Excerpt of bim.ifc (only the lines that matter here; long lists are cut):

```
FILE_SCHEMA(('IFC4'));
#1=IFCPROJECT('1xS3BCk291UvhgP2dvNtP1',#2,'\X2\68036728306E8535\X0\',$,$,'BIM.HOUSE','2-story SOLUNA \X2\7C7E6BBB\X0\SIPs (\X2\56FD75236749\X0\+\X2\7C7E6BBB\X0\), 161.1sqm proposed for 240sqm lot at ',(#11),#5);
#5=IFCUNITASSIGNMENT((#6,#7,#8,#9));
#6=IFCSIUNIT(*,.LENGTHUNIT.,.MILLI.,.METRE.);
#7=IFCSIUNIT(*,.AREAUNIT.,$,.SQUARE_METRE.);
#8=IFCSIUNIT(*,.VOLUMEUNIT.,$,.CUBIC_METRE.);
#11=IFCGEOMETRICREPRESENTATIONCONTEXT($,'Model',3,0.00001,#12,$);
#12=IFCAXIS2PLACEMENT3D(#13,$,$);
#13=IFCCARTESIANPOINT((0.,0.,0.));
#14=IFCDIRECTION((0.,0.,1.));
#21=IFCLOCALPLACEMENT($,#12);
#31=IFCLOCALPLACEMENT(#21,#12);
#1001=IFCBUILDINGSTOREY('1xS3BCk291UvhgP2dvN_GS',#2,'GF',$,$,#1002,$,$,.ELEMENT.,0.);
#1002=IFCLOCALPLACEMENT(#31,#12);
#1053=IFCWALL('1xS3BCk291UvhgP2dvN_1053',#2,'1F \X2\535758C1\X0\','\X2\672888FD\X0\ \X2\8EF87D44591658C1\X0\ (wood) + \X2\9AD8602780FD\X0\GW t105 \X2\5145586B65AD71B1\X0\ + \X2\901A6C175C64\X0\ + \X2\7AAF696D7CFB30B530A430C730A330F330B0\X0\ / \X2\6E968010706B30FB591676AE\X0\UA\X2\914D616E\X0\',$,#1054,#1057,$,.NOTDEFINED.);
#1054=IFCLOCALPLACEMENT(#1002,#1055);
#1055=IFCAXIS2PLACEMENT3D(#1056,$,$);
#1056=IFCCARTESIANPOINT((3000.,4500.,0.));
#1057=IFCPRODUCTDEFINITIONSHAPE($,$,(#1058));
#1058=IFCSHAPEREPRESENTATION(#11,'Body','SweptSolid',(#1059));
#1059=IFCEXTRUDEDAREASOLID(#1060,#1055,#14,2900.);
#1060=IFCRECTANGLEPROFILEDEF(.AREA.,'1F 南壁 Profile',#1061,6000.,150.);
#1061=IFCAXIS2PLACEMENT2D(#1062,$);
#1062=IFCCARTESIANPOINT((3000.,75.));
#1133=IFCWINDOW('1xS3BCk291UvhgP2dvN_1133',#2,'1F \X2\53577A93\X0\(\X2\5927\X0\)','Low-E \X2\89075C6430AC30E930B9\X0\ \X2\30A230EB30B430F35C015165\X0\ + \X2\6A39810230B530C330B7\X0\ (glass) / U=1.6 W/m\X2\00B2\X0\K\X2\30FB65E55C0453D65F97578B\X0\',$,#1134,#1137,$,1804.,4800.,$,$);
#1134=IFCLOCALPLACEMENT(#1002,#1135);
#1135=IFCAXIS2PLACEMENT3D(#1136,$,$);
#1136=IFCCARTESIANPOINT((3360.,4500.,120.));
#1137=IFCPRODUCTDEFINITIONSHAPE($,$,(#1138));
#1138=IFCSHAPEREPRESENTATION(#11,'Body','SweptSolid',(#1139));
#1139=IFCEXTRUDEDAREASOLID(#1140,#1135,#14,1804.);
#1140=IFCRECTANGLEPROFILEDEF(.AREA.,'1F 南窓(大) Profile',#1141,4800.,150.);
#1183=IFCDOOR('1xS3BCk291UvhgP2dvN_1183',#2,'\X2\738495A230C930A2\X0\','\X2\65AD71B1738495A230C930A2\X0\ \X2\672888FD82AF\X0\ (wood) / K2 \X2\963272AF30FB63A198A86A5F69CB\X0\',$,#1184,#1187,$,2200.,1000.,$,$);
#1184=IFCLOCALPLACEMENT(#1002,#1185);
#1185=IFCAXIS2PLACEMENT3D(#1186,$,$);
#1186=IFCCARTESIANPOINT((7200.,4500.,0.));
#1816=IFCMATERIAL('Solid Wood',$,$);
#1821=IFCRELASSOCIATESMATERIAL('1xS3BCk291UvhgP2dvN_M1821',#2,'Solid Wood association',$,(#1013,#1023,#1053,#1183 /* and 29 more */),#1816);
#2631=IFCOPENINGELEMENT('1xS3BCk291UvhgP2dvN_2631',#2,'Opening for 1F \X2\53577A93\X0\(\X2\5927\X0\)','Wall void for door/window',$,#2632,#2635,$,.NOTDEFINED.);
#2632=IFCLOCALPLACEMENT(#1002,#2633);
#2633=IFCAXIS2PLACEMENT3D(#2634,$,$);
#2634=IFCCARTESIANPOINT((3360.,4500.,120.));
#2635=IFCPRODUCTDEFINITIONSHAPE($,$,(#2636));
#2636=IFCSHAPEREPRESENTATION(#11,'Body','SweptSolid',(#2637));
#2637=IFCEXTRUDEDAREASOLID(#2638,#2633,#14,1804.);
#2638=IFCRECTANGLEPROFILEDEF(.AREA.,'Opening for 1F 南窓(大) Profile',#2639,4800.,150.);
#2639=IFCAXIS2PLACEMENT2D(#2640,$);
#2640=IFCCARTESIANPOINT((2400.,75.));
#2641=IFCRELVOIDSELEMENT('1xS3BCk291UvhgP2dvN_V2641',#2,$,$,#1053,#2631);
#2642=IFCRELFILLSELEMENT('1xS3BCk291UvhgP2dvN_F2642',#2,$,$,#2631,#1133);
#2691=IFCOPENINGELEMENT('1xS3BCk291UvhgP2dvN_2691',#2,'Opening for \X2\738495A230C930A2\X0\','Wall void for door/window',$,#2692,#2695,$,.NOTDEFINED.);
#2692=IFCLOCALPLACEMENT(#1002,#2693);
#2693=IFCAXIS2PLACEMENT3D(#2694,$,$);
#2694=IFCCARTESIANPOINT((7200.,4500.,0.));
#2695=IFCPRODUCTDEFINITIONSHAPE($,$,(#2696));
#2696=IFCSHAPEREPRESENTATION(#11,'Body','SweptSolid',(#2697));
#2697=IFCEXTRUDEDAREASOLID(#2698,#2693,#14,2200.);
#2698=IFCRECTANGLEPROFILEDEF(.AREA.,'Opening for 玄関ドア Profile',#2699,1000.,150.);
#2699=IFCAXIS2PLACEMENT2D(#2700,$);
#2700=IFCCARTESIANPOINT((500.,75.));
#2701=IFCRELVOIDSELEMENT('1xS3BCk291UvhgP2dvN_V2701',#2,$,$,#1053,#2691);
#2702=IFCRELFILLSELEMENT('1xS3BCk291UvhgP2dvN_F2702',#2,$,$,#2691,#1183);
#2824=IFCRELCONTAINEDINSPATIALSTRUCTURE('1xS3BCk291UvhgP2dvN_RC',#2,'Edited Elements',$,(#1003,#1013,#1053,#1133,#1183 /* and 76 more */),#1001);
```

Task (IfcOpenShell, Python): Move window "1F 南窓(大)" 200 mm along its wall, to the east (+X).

```python
import ifcopenshell
import ifcopenshell.api.geometry
import ifcopenshell.util.placement
import ifcopenshell.util.unit

model = ifcopenshell.open("bim.ifc")
unit_scale = ifcopenshell.util.unit.calculate_unit_scale(model)

window = model.by_guid("1xS3BCk291UvhgP2dvN_1133")
opening = window.FillsVoids[0].RelatingOpeningElement
wall = opening.VoidsElements[0].RelatingBuildingElement

wall_matrix = ifcopenshell.util.placement.get_local_placement(wall.ObjectPlacement)
shift = wall_matrix[:3, 0] * 0.2 / unit_scale
before = ifcopenshell.util.placement.get_local_placement(window.ObjectPlacement)[:3, 3].copy()

# The window is not placed relative to its opening, so move both.
for product in (opening, window):
    matrix = ifcopenshell.util.placement.get_local_placement(product.ObjectPlacement)
    matrix[:3, 3] += shift
    ifcopenshell.api.geometry.edit_object_placement(model, product=product, matrix=matrix, is_si=False)

after = ifcopenshell.util.placement.get_local_placement(window.ObjectPlacement)[:3, 3]
print("window moved by", (after - before).round(3) + 0.0)

model.write("bim_edited.ifc")
```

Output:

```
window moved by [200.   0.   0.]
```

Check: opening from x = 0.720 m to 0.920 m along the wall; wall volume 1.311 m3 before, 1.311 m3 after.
